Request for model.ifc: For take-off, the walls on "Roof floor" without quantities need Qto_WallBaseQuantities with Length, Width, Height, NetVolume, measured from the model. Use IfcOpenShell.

First a look at what the model holds.

```python
import ifcopenshell
import ifcopenshell.util.element
import ifcopenshell.util.unit

model = ifcopenshell.open("model.ifc")
print(model.schema)
for unit_type in ("LENGTHUNIT", "AREAUNIT", "VOLUMEUNIT"):
    print(unit_type, ifcopenshell.util.unit.calculate_unit_scale(model, unit_type))
storey = next(s for s in model.by_type("IfcBuildingStorey") if s.Name == "Roof floor")
walls = [e for e in ifcopenshell.util.element.get_decomposition(storey) if e.is_a("IfcWall")]
for e in sorted(walls, key=lambda e: e.id()):
    print(e.id(), e.is_a(), e.Name, list(ifcopenshell.util.element.get_psets(e, qtos_only=True)), sep=" | ")
```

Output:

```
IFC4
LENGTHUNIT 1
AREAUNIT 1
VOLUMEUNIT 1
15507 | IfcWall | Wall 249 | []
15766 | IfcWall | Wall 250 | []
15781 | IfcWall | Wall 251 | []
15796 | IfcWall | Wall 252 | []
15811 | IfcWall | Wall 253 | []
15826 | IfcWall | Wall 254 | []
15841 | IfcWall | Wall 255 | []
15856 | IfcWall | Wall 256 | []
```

```python
import ifcopenshell
import ifcopenshell.api.pset
import ifcopenshell.geom
import ifcopenshell.util.element
import ifcopenshell.util.shape
import ifcopenshell.util.unit

model = ifcopenshell.open("model.ifc")
unit_scale = ifcopenshell.util.unit.calculate_unit_scale(model)
volume_scale = ifcopenshell.util.unit.calculate_unit_scale(model, "VOLUMEUNIT")
settings = ifcopenshell.geom.settings()

storey = next(s for s in model.by_type("IfcBuildingStorey") if s.Name == "Roof floor")
walls = [e for e in ifcopenshell.util.element.get_decomposition(storey) if e.is_a("IfcWall")]

for e in sorted(walls, key=lambda e: e.id()):
    if ifcopenshell.util.element.get_psets(e, qtos_only=True, should_inherit=False):
        continue
    # Geometry comes back in metres, in the element's own axes.
    shape = ifcopenshell.geom.create_shape(settings, e)
    values = {
        "Length": ifcopenshell.util.shape.get_x(shape.geometry) / unit_scale,
        "Width": ifcopenshell.util.shape.get_y(shape.geometry) / unit_scale,
        "Height": ifcopenshell.util.shape.get_z(shape.geometry) / unit_scale,
        "NetVolume": ifcopenshell.util.shape.get_volume(shape.geometry) / volume_scale,
    }
    qto = ifcopenshell.api.pset.add_qto(model, product=e, name="Qto_WallBaseQuantities")
    ifcopenshell.api.pset.edit_qto(model, qto=qto, properties=values)
    print(e.id(), {k: round(v, 3) for k, v in values.items()})

model.write("model-out.ifc")
```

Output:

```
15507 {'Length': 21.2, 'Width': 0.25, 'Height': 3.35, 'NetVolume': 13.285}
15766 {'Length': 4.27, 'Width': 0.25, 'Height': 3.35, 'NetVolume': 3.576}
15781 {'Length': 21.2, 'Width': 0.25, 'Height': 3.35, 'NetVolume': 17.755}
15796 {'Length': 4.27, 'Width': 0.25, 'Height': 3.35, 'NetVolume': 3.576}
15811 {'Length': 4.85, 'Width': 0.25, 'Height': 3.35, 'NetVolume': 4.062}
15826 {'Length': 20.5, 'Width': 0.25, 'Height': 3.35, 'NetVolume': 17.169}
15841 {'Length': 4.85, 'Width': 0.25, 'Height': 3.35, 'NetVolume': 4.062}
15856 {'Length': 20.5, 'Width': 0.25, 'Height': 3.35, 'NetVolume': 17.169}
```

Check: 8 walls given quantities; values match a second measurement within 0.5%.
